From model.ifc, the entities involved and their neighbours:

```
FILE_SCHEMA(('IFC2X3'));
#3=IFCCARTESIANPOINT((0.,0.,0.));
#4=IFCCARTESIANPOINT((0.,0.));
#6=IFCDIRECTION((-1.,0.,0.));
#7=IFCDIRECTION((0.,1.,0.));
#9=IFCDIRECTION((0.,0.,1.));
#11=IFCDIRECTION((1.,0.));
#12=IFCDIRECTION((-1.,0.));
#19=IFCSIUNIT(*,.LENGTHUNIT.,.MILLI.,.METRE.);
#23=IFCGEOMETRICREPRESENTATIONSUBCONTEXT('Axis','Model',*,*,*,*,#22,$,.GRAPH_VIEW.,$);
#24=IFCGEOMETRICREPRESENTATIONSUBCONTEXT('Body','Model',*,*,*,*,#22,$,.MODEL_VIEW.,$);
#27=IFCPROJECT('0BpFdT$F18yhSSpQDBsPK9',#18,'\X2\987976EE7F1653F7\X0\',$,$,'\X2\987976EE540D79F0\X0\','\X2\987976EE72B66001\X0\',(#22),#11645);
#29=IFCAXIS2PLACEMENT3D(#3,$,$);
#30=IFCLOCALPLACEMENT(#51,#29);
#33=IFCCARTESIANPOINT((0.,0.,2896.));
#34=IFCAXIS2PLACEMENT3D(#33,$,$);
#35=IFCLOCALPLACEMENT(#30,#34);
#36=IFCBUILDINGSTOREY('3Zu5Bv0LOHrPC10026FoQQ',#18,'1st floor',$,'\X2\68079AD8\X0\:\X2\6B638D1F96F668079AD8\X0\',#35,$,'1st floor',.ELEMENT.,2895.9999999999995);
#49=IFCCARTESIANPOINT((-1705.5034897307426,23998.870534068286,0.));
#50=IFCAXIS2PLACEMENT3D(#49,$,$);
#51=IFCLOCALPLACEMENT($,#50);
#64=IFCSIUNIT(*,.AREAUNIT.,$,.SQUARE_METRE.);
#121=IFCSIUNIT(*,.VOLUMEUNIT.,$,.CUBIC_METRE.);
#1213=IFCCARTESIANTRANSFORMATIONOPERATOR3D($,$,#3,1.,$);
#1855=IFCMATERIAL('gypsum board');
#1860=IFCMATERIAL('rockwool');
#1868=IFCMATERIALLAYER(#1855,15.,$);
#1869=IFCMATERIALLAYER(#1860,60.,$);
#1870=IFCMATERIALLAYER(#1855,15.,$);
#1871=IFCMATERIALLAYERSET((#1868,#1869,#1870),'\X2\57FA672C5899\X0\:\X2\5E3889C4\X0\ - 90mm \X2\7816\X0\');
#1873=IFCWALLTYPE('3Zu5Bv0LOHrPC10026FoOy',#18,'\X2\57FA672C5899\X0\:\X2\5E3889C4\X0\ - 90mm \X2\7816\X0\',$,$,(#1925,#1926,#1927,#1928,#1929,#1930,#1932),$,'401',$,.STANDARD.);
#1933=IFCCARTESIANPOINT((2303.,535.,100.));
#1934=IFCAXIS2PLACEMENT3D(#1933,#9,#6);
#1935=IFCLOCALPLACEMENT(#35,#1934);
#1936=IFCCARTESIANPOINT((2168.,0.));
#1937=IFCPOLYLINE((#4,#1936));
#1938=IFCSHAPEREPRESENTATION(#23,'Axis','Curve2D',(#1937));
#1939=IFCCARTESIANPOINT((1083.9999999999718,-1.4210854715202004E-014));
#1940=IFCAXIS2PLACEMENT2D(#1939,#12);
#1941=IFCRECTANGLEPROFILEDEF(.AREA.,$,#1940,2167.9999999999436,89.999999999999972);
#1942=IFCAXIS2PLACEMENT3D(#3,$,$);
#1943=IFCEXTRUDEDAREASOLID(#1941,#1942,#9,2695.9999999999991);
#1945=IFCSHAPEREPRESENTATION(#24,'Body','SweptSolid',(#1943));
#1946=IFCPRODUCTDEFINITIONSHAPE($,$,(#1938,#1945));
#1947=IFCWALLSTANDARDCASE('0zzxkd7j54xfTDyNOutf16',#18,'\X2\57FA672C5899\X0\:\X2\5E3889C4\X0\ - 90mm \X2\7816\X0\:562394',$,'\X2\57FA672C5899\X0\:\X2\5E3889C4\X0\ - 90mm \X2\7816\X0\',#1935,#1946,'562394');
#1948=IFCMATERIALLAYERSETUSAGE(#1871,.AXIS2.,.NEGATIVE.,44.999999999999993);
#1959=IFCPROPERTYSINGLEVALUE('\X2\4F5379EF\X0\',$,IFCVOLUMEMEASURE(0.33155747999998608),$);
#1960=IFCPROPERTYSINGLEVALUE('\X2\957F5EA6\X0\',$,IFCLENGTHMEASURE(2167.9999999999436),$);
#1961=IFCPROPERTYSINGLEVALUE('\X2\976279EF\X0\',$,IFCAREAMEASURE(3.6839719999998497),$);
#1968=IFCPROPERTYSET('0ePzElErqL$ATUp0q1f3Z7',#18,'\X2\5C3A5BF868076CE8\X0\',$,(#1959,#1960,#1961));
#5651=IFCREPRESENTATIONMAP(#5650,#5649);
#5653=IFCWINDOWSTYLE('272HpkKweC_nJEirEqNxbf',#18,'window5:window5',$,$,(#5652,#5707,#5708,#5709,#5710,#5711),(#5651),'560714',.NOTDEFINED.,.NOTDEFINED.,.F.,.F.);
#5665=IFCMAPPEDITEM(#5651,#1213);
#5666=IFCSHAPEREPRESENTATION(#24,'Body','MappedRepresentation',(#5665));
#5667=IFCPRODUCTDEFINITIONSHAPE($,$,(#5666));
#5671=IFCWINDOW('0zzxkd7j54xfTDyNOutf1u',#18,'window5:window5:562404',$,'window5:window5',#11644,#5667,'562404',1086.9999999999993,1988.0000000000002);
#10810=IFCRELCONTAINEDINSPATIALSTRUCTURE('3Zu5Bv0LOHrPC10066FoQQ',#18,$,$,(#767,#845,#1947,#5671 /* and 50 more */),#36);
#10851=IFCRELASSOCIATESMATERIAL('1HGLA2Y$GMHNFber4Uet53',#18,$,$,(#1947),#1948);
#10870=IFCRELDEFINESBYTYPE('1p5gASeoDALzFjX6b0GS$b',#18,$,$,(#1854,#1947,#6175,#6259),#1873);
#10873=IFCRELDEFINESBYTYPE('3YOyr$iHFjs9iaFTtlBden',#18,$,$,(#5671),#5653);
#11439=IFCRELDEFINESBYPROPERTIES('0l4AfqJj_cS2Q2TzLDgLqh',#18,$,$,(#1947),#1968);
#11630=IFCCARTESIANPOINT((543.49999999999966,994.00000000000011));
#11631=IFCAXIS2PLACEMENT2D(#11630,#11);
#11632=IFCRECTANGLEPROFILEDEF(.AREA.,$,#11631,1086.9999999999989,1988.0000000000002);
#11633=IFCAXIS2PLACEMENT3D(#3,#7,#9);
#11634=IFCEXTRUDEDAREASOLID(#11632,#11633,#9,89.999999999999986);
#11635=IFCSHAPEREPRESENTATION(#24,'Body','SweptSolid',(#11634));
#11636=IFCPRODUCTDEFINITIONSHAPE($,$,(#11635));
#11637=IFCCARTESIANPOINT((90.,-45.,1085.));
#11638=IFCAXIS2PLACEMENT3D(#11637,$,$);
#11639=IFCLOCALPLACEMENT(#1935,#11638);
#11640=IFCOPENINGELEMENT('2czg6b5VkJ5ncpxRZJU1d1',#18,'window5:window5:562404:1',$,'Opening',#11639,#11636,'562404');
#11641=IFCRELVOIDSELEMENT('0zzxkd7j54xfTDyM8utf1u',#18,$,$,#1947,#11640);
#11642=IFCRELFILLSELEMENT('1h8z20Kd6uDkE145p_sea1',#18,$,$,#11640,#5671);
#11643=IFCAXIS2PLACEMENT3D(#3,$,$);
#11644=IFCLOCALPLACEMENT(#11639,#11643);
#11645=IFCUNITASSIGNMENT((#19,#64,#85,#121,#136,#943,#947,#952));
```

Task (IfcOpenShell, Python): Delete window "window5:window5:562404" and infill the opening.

```python
import ifcopenshell
import ifcopenshell.api.feature
import ifcopenshell.api.pset
import ifcopenshell.api.root
import ifcopenshell.geom
import ifcopenshell.util.element
import ifcopenshell.util.shape
import ifcopenshell.util.unit

model = ifcopenshell.open("model.ifc")
area_scale = ifcopenshell.util.unit.calculate_unit_scale(model, "AREAUNIT")
volume_scale = ifcopenshell.util.unit.calculate_unit_scale(model, "VOLUMEUNIT")
settings = ifcopenshell.geom.settings()


def volume(element):
    """Net volume in cubic metres, openings subtracted."""
    shape = ifcopenshell.geom.create_shape(settings, element)
    return ifcopenshell.util.shape.get_volume(shape.geometry)


window = model.by_id(5671)
opening = window.FillsVoids[0].RelatingOpeningElement
wall = opening.VoidsElements[0].RelatingBuildingElement
before = volume(wall)

ifcopenshell.api.root.remove_product(model, product=window)
ifcopenshell.api.feature.remove_feature(model, feature=opening)

after = volume(wall)
thickness = 0.09  # wall thickness in metres

# Update the wall's stored quantities.
pset = model.by_id(ifcopenshell.util.element.get_pset(wall, "尺寸标注", should_inherit=False)["id"])
ifcopenshell.api.pset.edit_pset(model, pset=pset, properties={
    "体积": model.create_entity("IfcVolumeMeasure", after / volume_scale),
    "面积": model.create_entity("IfcAreaMeasure", after / thickness / area_scale),
})

print(f"wall volume {before:.3f} -> {after:.3f} m3")

model.write("model_rev.ifc")
```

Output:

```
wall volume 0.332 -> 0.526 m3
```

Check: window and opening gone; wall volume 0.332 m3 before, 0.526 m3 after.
